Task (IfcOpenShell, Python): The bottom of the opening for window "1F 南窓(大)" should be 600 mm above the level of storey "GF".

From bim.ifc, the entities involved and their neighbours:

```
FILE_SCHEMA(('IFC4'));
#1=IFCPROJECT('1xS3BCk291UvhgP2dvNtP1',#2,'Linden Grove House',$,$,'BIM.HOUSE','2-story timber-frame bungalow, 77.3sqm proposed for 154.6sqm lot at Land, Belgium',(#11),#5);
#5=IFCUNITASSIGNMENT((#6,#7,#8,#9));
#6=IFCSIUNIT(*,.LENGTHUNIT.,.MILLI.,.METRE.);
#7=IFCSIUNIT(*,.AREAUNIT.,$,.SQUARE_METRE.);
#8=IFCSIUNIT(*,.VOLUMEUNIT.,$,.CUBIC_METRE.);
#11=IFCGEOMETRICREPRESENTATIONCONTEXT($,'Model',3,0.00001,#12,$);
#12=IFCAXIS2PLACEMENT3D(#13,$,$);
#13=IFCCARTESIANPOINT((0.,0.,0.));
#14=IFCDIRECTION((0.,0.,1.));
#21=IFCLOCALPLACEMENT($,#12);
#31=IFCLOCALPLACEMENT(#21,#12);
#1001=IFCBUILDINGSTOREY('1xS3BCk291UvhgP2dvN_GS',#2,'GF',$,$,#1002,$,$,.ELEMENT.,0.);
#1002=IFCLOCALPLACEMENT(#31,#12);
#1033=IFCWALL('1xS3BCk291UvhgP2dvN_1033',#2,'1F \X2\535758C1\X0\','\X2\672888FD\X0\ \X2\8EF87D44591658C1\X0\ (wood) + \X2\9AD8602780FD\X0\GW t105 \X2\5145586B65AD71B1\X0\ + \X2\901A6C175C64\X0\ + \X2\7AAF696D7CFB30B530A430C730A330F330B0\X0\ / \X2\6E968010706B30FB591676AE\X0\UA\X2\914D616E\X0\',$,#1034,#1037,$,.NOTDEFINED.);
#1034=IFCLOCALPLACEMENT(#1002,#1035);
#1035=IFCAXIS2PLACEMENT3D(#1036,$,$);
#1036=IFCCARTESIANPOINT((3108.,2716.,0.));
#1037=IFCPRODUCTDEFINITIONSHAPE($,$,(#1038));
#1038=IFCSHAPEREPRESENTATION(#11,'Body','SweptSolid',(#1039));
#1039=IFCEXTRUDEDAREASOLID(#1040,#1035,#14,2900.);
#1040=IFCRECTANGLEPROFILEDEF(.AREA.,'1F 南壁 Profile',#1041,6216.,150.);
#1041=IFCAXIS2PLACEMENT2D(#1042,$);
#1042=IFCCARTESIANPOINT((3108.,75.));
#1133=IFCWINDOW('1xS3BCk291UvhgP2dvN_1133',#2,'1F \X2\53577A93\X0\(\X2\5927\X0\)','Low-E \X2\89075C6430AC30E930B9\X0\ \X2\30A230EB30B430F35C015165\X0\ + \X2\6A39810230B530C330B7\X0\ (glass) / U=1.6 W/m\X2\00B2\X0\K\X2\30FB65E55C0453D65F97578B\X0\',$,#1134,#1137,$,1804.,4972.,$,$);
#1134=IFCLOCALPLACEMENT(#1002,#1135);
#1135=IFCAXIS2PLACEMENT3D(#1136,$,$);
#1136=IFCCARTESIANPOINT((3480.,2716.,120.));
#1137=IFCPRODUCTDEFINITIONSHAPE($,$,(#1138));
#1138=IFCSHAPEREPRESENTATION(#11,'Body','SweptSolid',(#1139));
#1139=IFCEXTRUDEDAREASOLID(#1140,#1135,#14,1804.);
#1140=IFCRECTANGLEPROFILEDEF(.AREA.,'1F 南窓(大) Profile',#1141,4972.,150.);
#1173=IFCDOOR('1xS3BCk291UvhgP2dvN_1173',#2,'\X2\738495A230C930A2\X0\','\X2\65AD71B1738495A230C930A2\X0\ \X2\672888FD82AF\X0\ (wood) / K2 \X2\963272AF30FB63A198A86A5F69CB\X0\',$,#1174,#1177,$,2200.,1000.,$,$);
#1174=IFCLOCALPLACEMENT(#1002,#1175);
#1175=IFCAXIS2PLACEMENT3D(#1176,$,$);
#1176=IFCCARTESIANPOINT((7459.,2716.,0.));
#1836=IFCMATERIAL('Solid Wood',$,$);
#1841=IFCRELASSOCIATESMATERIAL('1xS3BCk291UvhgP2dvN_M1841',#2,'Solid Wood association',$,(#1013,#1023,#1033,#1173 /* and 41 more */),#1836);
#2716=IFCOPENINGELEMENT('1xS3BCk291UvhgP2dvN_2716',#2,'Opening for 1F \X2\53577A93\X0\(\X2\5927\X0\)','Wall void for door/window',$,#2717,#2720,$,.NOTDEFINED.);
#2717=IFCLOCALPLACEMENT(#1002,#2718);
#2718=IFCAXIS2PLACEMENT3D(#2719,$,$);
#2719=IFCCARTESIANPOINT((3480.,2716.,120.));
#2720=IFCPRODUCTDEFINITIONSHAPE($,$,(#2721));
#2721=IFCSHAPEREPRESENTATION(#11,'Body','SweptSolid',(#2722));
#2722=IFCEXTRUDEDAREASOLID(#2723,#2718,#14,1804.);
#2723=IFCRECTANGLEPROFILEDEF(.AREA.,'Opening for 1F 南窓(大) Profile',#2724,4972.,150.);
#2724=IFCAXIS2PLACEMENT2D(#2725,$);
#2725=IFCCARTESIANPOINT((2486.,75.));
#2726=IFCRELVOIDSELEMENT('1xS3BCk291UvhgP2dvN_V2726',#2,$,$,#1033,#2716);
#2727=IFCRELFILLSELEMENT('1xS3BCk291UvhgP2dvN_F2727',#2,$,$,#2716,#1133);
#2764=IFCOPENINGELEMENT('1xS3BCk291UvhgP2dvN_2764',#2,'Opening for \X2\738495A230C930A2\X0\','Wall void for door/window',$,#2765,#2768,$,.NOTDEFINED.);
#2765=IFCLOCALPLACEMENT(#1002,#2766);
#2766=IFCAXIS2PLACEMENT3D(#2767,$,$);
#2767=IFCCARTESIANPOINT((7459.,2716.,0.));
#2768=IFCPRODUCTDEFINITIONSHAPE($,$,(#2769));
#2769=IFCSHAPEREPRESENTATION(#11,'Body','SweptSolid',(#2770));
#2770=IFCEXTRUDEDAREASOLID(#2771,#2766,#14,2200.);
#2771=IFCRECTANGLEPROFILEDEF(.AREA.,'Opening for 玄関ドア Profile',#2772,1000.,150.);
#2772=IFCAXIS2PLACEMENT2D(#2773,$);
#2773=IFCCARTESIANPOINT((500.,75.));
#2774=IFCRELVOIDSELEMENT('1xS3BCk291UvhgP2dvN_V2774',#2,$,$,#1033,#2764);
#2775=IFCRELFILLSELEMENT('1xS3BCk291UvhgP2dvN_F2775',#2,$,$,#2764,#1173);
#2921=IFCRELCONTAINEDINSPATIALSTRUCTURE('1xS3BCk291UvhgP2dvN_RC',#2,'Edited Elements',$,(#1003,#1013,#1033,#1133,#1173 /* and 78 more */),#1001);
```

```python
import numpy as np
import ifcopenshell
import ifcopenshell.api.geometry
import ifcopenshell.geom
import ifcopenshell.util.element
import ifcopenshell.util.placement
import ifcopenshell.util.shape
import ifcopenshell.util.unit

model = ifcopenshell.open("bim.ifc")
unit_scale = ifcopenshell.util.unit.calculate_unit_scale(model)

window = model.by_id(1133)
opening = window.FillsVoids[0].RelatingOpeningElement
storey = ifcopenshell.util.element.get_container(window, ifc_class="IfcBuildingStorey")
level = ifcopenshell.util.placement.get_local_placement(storey.ObjectPlacement)[2, 3]

# The opening's origin need not be at the sill, so measure its lowest point.
shape = ifcopenshell.geom.create_shape(ifcopenshell.geom.settings(), opening)
bottom = ifcopenshell.util.shape.get_shape_bottom_elevation(shape, shape.geometry) / unit_scale
dz = level + 600.0 - bottom

shift = np.array([0.0, 0.0, dz])
# The window is not placed relative to its opening, so move both.
for product in (opening, window):
    matrix = ifcopenshell.util.placement.get_local_placement(product.ObjectPlacement)
    matrix[:3, 3] += shift
    ifcopenshell.api.geometry.edit_object_placement(model, product=product, matrix=matrix, is_si=False)

print(f"moved by {dz * unit_scale:+.3f} m")

model.write("bim_rev.ifc")
```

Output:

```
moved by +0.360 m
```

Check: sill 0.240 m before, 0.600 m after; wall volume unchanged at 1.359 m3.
